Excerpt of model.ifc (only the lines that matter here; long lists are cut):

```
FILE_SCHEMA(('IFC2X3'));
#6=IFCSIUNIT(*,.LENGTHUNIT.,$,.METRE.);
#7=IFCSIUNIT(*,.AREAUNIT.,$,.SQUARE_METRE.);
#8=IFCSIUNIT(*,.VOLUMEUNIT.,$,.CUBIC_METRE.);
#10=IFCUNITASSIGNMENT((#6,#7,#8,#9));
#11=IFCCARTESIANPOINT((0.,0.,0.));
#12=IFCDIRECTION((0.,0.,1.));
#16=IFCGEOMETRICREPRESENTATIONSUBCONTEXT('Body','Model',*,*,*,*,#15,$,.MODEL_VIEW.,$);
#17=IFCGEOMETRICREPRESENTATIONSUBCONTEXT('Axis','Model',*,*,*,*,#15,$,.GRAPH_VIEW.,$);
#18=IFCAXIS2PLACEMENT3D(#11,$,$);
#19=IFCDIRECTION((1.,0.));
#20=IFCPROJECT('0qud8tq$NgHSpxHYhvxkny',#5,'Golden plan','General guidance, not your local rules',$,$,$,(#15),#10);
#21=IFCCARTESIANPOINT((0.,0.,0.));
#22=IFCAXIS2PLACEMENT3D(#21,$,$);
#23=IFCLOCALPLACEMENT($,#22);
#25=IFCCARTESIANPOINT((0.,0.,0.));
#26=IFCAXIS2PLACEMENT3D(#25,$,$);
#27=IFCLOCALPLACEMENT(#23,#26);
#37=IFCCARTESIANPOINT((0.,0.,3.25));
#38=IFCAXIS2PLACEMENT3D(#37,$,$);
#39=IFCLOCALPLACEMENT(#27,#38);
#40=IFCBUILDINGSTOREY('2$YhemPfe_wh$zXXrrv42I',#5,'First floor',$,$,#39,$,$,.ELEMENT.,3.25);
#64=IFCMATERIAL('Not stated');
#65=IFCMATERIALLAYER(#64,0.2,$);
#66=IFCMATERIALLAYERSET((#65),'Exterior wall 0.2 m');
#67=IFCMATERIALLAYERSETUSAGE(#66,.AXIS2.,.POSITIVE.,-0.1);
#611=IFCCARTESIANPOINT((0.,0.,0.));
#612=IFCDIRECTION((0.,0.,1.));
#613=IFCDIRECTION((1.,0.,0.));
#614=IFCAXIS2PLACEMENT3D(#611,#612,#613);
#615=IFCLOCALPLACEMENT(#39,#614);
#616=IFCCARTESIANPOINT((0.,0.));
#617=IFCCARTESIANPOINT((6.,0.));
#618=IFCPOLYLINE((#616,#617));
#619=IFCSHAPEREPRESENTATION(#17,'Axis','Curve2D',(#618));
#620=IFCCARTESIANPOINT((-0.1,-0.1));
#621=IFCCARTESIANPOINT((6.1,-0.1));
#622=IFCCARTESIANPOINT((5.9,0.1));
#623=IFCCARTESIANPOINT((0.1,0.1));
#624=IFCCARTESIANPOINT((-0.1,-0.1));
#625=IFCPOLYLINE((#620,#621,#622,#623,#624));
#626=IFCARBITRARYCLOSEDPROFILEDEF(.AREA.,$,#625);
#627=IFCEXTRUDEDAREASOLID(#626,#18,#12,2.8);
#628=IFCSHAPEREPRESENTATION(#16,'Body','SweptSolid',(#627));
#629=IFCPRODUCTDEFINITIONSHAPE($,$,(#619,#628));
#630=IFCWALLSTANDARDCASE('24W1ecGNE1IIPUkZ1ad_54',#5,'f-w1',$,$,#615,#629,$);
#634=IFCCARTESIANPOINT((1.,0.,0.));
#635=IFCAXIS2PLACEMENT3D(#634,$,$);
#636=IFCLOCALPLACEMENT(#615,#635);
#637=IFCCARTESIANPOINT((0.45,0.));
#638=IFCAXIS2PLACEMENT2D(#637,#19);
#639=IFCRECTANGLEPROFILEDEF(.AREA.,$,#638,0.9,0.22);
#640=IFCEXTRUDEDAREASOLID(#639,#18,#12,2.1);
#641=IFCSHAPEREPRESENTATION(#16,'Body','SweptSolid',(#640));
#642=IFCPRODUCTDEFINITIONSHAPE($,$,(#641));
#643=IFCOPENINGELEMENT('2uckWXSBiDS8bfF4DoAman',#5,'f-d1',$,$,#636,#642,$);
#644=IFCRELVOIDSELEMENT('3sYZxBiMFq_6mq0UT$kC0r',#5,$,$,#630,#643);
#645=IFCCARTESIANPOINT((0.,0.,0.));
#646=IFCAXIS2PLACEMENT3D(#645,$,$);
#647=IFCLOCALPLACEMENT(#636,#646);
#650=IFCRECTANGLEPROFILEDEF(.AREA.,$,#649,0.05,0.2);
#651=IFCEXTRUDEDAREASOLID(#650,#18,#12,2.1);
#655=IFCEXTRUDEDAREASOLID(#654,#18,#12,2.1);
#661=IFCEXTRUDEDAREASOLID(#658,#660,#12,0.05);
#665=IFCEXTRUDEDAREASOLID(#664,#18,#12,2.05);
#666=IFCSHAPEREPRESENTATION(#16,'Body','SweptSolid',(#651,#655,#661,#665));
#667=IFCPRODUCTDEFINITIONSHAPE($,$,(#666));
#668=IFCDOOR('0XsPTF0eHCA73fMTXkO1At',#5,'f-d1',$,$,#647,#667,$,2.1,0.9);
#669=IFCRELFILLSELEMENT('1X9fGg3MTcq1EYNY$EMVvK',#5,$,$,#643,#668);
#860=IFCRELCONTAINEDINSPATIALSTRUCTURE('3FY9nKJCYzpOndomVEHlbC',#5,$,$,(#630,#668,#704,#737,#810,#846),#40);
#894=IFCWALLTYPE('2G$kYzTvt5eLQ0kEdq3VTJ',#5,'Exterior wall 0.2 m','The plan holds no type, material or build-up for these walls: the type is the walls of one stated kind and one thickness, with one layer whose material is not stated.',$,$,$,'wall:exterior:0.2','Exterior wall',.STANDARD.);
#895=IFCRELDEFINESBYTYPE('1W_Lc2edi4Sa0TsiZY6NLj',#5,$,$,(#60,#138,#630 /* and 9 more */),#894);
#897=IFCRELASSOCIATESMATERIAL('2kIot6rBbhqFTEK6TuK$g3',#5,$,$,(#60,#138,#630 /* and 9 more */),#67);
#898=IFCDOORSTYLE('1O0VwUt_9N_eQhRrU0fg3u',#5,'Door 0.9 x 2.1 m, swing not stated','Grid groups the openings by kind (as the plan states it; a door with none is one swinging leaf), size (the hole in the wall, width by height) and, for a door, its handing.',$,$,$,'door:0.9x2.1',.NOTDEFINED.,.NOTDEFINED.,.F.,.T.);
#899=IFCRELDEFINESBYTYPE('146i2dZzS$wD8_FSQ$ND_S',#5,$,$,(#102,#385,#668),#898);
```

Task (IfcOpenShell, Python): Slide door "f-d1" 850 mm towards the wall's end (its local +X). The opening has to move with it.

```python
import ifcopenshell
import ifcopenshell.api.geometry
import ifcopenshell.util.placement
import ifcopenshell.util.unit

model = ifcopenshell.open("model.ifc")
unit_scale = ifcopenshell.util.unit.calculate_unit_scale(model)

door = model.by_guid("0XsPTF0eHCA73fMTXkO1At")
opening = door.FillsVoids[0].RelatingOpeningElement
wall = opening.VoidsElements[0].RelatingBuildingElement

wall_matrix = ifcopenshell.util.placement.get_local_placement(wall.ObjectPlacement)
shift = wall_matrix[:3, 0] * 0.85 / unit_scale
before = ifcopenshell.util.placement.get_local_placement(door.ObjectPlacement)[:3, 3].copy()

# The door is placed relative to its opening, so it follows when the opening moves.
matrix = ifcopenshell.util.placement.get_local_placement(opening.ObjectPlacement)
matrix[:3, 3] += shift
ifcopenshell.api.geometry.edit_object_placement(
    model, product=opening, matrix=matrix, is_si=False, should_transform_children=True
)

after = ifcopenshell.util.placement.get_local_placement(door.ObjectPlacement)[:3, 3]
print("door moved by", (after - before).round(3) + 0.0)

model.write("model_edited.ifc")
```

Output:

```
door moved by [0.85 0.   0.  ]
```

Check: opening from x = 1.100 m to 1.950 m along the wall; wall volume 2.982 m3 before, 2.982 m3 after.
